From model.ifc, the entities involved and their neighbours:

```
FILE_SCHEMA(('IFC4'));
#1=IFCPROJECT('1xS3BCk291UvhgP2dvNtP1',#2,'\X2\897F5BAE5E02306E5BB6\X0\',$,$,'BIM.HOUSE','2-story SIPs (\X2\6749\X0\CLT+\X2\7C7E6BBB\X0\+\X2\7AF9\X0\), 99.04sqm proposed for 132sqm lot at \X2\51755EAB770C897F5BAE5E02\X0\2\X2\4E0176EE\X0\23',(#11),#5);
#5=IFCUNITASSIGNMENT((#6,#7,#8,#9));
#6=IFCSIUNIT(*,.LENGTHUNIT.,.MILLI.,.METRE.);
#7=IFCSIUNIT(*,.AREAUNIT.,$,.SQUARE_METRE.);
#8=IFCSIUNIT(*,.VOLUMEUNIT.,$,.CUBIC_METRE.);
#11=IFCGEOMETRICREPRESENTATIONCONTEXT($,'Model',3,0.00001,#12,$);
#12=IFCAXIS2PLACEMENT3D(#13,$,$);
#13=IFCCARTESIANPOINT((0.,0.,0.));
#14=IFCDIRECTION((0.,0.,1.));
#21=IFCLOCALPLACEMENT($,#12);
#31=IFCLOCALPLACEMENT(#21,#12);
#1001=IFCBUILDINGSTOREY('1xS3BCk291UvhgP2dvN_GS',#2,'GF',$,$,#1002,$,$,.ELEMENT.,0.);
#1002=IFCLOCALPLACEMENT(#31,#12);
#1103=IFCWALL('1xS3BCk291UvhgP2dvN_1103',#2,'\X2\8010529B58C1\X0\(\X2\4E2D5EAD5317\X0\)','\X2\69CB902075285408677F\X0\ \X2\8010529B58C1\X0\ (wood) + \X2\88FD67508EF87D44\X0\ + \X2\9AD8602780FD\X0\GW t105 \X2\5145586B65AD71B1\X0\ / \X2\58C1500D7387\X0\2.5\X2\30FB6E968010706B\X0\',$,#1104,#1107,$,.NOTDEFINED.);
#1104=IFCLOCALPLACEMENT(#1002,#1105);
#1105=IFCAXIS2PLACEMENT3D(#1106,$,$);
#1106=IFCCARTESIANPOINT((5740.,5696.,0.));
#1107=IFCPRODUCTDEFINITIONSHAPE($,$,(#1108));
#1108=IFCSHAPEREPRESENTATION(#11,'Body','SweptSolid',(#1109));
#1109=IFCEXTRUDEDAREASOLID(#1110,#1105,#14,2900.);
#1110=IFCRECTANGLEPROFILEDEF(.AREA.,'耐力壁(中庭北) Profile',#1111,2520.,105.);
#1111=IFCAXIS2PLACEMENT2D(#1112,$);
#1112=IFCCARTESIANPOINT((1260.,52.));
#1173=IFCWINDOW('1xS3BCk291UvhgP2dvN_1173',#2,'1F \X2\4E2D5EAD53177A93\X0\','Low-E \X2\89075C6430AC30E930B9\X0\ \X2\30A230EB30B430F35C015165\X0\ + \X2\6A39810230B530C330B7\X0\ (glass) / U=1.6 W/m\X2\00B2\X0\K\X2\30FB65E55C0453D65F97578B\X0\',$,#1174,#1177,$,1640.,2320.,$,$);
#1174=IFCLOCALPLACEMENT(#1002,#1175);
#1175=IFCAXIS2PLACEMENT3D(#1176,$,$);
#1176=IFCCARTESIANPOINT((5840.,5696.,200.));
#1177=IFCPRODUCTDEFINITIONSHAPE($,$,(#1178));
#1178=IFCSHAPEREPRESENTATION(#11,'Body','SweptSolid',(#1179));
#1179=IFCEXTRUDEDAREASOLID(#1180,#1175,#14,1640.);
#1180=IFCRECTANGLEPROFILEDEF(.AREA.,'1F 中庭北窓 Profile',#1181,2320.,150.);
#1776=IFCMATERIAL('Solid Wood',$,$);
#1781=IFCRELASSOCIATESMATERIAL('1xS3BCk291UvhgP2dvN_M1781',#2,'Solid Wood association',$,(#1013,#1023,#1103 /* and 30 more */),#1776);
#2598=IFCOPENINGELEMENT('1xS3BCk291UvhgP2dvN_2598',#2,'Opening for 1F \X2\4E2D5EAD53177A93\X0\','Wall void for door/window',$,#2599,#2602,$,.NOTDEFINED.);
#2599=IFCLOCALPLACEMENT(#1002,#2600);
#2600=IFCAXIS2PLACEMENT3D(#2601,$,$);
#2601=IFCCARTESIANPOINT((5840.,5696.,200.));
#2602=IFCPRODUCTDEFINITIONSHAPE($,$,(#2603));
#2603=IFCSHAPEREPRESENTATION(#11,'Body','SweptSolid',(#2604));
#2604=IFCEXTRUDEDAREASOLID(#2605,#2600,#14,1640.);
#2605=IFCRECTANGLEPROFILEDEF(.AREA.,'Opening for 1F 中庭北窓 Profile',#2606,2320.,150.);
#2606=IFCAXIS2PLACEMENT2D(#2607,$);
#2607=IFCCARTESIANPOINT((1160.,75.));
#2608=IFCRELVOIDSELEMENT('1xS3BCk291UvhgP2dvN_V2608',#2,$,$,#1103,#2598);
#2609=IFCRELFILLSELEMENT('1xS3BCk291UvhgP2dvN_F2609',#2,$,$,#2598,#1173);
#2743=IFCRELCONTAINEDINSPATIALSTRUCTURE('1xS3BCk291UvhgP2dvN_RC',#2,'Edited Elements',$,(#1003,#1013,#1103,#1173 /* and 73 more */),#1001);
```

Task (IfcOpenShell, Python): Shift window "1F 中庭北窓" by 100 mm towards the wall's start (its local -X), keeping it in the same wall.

```python
import ifcopenshell
import ifcopenshell.api.geometry
import ifcopenshell.util.placement

model = ifcopenshell.open("model.ifc")

window = model.by_guid("1xS3BCk291UvhgP2dvN_1173")
opening = window.FillsVoids[0].RelatingOpeningElement
wall = opening.VoidsElements[0].RelatingBuildingElement

wall_matrix = ifcopenshell.util.placement.get_local_placement(wall.ObjectPlacement)
shift = wall_matrix[:3, 0] * -100.0
before = ifcopenshell.util.placement.get_local_placement(window.ObjectPlacement)[:3, 3].copy()

# The window is not placed relative to its opening, so move both.
for product in (opening, window):
    matrix = ifcopenshell.util.placement.get_local_placement(product.ObjectPlacement)
    matrix[:3, 3] += shift
    ifcopenshell.api.geometry.edit_object_placement(model, product=product, matrix=matrix, is_si=False)

after = ifcopenshell.util.placement.get_local_placement(window.ObjectPlacement)[:3, 3]
print("window moved by", (after - before).round(3) + 0.0)

model.write("model_edited.ifc")
```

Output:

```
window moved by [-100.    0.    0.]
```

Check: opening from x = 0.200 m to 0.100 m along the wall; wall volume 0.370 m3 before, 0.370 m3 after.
